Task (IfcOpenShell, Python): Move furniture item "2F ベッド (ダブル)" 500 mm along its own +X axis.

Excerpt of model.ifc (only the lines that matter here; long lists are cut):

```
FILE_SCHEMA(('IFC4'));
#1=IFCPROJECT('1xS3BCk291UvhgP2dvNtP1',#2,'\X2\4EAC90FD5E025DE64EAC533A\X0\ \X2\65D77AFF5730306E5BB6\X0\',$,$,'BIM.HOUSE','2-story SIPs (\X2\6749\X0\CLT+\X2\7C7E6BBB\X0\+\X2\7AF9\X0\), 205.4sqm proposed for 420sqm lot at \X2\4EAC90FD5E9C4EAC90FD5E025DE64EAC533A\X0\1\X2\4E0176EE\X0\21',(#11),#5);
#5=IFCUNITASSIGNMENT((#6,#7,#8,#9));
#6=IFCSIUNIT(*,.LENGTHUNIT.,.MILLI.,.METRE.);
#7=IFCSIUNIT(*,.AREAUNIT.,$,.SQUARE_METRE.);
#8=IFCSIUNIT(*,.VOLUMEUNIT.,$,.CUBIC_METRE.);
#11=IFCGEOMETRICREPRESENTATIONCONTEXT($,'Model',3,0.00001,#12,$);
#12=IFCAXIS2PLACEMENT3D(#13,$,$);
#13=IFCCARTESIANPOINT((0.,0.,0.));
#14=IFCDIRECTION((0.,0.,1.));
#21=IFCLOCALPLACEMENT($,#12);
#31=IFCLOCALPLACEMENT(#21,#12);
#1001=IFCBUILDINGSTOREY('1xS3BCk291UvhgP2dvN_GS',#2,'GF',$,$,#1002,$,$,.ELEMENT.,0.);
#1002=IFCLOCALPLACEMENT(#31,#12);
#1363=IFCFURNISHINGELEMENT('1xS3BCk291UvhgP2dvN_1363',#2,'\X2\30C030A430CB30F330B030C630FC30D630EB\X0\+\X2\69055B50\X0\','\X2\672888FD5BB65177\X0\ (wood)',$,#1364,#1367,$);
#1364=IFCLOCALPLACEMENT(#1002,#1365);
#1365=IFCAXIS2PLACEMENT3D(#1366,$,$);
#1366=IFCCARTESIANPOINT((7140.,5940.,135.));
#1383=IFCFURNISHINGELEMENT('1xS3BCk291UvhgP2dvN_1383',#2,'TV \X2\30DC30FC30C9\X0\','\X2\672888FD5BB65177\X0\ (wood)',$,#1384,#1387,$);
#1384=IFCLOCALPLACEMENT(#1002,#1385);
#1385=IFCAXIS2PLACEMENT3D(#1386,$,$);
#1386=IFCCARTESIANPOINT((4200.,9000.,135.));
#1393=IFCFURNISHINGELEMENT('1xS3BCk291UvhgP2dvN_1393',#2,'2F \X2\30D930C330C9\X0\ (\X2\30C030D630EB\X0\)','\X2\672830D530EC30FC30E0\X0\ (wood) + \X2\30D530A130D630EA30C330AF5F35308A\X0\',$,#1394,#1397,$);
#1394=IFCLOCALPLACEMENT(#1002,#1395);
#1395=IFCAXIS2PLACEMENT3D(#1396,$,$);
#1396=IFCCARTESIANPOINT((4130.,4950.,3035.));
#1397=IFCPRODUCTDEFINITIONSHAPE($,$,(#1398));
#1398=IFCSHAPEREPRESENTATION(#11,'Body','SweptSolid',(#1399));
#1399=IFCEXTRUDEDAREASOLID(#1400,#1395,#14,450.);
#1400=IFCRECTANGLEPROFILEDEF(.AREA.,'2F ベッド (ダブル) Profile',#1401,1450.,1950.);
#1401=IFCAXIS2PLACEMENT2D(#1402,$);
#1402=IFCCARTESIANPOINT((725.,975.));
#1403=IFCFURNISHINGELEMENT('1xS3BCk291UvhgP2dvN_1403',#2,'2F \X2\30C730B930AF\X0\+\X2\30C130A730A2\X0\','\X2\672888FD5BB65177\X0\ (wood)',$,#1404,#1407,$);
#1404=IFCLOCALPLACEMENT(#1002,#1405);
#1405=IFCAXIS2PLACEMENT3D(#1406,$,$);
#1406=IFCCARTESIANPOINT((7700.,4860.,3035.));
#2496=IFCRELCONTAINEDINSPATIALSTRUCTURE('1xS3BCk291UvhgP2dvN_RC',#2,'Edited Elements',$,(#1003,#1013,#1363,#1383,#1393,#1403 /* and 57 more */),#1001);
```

```python
import ifcopenshell
import ifcopenshell.api.geometry
import ifcopenshell.util.placement

model = ifcopenshell.open("model.ifc")

item = model.by_id(1393)
matrix = ifcopenshell.util.placement.get_local_placement(item.ObjectPlacement)
matrix[:3, 3] += matrix[:3, 0] * 500.0
ifcopenshell.api.geometry.edit_object_placement(model, product=item, matrix=matrix, is_si=False)

print(ifcopenshell.util.placement.get_local_placement(item.ObjectPlacement).round(3) + 0.0)

model.write("model_rev.ifc")
```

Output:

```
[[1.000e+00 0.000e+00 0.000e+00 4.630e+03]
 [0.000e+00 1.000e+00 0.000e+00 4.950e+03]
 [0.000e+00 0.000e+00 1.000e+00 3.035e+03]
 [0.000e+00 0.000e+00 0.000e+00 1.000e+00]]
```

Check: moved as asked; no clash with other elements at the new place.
